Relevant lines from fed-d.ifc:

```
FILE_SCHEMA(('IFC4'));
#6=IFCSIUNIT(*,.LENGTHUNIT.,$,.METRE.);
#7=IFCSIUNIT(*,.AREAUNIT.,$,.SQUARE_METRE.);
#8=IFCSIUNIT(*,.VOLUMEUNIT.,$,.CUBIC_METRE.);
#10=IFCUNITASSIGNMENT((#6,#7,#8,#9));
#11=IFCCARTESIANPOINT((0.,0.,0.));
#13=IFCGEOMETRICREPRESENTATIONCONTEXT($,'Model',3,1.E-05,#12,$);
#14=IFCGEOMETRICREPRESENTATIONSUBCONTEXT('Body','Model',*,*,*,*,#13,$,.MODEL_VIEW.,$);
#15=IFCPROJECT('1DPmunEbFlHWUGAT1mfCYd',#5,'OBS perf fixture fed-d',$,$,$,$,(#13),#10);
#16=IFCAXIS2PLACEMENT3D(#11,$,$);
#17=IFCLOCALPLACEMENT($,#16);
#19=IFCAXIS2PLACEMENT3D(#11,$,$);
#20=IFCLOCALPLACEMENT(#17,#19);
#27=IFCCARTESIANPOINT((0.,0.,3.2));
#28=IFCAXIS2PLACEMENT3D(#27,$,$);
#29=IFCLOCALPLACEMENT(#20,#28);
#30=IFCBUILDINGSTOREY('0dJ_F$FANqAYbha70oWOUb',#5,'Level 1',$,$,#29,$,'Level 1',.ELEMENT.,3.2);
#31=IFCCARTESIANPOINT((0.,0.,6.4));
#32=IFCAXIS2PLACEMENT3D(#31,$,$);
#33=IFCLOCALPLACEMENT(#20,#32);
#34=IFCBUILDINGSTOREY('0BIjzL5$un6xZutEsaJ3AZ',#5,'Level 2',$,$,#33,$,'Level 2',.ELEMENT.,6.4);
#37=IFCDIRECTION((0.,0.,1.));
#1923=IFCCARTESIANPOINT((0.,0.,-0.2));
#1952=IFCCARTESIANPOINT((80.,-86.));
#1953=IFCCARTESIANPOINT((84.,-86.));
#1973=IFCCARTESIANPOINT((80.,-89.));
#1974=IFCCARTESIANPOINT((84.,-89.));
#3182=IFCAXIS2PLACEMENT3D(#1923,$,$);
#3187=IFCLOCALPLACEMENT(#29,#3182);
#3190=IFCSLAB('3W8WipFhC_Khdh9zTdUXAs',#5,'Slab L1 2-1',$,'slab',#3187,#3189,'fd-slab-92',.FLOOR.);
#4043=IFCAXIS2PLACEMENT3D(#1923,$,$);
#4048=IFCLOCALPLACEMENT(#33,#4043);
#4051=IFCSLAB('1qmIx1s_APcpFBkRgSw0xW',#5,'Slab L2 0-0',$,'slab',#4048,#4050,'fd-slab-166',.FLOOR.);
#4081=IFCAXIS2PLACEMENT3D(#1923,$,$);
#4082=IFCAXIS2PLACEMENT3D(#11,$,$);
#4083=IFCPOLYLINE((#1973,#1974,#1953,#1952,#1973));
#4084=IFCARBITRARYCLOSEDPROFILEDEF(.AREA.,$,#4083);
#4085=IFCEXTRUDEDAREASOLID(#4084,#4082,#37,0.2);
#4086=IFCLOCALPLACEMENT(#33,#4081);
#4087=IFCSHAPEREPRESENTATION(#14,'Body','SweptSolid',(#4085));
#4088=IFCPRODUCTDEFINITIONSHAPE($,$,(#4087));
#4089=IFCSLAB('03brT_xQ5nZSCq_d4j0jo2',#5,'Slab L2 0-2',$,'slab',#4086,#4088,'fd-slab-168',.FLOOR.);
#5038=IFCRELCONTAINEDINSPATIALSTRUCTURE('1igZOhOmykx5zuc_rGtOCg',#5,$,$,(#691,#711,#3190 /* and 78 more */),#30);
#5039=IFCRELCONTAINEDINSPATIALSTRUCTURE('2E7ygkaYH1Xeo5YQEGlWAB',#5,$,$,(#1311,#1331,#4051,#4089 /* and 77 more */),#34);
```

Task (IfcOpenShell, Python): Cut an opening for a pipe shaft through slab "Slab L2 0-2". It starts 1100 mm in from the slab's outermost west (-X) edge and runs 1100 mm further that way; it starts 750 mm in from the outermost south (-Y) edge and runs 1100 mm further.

```python
import numpy as np
import ifcopenshell
import ifcopenshell.api.feature
import ifcopenshell.api.geometry
import ifcopenshell.api.root
import ifcopenshell.geom
import ifcopenshell.util.placement
import ifcopenshell.util.representation
import ifcopenshell.util.shape
import ifcopenshell.util.unit

model = ifcopenshell.open("fed-d.ifc")
unit_scale = ifcopenshell.util.unit.calculate_unit_scale(model)
settings = ifcopenshell.geom.settings()


def volume(element):
    """Net volume in cubic metres, openings subtracted."""
    shape = ifcopenshell.geom.create_shape(settings, element)
    return ifcopenshell.util.shape.get_volume(shape.geometry)


slab = model.by_guid("03brT_xQ5nZSCq_d4j0jo2")
before = volume(slab)

# Extent in the slab's own axes, in metres. The edges named are its -X and -Y sides.
slab_shape = ifcopenshell.geom.create_shape(settings, slab)
vertices = ifcopenshell.util.shape.get_vertices(slab_shape.geometry)
x_min, y_min, bottom = vertices.min(axis=0)
top = vertices[:, 2].max()

opening = ifcopenshell.api.root.create_entity(model, ifc_class="IfcOpeningElement", name="Pipe shaft opening", predefined_type="OPENING")
context = ifcopenshell.util.representation.get_context(model, "Model", "Body", "MODEL_VIEW")
width, depth = 1.1, 1.1
outline = [(0.0, 0.0), (width, 0.0), (width, depth), (0.0, depth), (0.0, 0.0)]
# Overshoot both faces by 50 mm so the cut is clean.
shape = ifcopenshell.api.geometry.add_slab_representation(
    model, context=context, depth=top - bottom + 0.1, polyline=outline
)
ifcopenshell.api.geometry.assign_representation(model, product=opening, representation=shape)

matrix = ifcopenshell.util.placement.get_local_placement(slab.ObjectPlacement)
matrix[:, 3] = matrix @ np.append(np.array([x_min + 1.1, y_min + 0.75, bottom - 0.05]) / unit_scale, 1.0)
ifcopenshell.api.geometry.edit_object_placement(model, product=opening, matrix=matrix, is_si=False)
ifcopenshell.api.feature.add_feature(model, feature=opening, element=slab)

after = volume(slab)

print(f"slab volume {before:.3f} -> {after:.3f} m3")

model.write("fed-d_edited.ifc")
```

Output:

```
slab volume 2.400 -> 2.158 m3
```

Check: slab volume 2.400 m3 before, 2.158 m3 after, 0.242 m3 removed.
